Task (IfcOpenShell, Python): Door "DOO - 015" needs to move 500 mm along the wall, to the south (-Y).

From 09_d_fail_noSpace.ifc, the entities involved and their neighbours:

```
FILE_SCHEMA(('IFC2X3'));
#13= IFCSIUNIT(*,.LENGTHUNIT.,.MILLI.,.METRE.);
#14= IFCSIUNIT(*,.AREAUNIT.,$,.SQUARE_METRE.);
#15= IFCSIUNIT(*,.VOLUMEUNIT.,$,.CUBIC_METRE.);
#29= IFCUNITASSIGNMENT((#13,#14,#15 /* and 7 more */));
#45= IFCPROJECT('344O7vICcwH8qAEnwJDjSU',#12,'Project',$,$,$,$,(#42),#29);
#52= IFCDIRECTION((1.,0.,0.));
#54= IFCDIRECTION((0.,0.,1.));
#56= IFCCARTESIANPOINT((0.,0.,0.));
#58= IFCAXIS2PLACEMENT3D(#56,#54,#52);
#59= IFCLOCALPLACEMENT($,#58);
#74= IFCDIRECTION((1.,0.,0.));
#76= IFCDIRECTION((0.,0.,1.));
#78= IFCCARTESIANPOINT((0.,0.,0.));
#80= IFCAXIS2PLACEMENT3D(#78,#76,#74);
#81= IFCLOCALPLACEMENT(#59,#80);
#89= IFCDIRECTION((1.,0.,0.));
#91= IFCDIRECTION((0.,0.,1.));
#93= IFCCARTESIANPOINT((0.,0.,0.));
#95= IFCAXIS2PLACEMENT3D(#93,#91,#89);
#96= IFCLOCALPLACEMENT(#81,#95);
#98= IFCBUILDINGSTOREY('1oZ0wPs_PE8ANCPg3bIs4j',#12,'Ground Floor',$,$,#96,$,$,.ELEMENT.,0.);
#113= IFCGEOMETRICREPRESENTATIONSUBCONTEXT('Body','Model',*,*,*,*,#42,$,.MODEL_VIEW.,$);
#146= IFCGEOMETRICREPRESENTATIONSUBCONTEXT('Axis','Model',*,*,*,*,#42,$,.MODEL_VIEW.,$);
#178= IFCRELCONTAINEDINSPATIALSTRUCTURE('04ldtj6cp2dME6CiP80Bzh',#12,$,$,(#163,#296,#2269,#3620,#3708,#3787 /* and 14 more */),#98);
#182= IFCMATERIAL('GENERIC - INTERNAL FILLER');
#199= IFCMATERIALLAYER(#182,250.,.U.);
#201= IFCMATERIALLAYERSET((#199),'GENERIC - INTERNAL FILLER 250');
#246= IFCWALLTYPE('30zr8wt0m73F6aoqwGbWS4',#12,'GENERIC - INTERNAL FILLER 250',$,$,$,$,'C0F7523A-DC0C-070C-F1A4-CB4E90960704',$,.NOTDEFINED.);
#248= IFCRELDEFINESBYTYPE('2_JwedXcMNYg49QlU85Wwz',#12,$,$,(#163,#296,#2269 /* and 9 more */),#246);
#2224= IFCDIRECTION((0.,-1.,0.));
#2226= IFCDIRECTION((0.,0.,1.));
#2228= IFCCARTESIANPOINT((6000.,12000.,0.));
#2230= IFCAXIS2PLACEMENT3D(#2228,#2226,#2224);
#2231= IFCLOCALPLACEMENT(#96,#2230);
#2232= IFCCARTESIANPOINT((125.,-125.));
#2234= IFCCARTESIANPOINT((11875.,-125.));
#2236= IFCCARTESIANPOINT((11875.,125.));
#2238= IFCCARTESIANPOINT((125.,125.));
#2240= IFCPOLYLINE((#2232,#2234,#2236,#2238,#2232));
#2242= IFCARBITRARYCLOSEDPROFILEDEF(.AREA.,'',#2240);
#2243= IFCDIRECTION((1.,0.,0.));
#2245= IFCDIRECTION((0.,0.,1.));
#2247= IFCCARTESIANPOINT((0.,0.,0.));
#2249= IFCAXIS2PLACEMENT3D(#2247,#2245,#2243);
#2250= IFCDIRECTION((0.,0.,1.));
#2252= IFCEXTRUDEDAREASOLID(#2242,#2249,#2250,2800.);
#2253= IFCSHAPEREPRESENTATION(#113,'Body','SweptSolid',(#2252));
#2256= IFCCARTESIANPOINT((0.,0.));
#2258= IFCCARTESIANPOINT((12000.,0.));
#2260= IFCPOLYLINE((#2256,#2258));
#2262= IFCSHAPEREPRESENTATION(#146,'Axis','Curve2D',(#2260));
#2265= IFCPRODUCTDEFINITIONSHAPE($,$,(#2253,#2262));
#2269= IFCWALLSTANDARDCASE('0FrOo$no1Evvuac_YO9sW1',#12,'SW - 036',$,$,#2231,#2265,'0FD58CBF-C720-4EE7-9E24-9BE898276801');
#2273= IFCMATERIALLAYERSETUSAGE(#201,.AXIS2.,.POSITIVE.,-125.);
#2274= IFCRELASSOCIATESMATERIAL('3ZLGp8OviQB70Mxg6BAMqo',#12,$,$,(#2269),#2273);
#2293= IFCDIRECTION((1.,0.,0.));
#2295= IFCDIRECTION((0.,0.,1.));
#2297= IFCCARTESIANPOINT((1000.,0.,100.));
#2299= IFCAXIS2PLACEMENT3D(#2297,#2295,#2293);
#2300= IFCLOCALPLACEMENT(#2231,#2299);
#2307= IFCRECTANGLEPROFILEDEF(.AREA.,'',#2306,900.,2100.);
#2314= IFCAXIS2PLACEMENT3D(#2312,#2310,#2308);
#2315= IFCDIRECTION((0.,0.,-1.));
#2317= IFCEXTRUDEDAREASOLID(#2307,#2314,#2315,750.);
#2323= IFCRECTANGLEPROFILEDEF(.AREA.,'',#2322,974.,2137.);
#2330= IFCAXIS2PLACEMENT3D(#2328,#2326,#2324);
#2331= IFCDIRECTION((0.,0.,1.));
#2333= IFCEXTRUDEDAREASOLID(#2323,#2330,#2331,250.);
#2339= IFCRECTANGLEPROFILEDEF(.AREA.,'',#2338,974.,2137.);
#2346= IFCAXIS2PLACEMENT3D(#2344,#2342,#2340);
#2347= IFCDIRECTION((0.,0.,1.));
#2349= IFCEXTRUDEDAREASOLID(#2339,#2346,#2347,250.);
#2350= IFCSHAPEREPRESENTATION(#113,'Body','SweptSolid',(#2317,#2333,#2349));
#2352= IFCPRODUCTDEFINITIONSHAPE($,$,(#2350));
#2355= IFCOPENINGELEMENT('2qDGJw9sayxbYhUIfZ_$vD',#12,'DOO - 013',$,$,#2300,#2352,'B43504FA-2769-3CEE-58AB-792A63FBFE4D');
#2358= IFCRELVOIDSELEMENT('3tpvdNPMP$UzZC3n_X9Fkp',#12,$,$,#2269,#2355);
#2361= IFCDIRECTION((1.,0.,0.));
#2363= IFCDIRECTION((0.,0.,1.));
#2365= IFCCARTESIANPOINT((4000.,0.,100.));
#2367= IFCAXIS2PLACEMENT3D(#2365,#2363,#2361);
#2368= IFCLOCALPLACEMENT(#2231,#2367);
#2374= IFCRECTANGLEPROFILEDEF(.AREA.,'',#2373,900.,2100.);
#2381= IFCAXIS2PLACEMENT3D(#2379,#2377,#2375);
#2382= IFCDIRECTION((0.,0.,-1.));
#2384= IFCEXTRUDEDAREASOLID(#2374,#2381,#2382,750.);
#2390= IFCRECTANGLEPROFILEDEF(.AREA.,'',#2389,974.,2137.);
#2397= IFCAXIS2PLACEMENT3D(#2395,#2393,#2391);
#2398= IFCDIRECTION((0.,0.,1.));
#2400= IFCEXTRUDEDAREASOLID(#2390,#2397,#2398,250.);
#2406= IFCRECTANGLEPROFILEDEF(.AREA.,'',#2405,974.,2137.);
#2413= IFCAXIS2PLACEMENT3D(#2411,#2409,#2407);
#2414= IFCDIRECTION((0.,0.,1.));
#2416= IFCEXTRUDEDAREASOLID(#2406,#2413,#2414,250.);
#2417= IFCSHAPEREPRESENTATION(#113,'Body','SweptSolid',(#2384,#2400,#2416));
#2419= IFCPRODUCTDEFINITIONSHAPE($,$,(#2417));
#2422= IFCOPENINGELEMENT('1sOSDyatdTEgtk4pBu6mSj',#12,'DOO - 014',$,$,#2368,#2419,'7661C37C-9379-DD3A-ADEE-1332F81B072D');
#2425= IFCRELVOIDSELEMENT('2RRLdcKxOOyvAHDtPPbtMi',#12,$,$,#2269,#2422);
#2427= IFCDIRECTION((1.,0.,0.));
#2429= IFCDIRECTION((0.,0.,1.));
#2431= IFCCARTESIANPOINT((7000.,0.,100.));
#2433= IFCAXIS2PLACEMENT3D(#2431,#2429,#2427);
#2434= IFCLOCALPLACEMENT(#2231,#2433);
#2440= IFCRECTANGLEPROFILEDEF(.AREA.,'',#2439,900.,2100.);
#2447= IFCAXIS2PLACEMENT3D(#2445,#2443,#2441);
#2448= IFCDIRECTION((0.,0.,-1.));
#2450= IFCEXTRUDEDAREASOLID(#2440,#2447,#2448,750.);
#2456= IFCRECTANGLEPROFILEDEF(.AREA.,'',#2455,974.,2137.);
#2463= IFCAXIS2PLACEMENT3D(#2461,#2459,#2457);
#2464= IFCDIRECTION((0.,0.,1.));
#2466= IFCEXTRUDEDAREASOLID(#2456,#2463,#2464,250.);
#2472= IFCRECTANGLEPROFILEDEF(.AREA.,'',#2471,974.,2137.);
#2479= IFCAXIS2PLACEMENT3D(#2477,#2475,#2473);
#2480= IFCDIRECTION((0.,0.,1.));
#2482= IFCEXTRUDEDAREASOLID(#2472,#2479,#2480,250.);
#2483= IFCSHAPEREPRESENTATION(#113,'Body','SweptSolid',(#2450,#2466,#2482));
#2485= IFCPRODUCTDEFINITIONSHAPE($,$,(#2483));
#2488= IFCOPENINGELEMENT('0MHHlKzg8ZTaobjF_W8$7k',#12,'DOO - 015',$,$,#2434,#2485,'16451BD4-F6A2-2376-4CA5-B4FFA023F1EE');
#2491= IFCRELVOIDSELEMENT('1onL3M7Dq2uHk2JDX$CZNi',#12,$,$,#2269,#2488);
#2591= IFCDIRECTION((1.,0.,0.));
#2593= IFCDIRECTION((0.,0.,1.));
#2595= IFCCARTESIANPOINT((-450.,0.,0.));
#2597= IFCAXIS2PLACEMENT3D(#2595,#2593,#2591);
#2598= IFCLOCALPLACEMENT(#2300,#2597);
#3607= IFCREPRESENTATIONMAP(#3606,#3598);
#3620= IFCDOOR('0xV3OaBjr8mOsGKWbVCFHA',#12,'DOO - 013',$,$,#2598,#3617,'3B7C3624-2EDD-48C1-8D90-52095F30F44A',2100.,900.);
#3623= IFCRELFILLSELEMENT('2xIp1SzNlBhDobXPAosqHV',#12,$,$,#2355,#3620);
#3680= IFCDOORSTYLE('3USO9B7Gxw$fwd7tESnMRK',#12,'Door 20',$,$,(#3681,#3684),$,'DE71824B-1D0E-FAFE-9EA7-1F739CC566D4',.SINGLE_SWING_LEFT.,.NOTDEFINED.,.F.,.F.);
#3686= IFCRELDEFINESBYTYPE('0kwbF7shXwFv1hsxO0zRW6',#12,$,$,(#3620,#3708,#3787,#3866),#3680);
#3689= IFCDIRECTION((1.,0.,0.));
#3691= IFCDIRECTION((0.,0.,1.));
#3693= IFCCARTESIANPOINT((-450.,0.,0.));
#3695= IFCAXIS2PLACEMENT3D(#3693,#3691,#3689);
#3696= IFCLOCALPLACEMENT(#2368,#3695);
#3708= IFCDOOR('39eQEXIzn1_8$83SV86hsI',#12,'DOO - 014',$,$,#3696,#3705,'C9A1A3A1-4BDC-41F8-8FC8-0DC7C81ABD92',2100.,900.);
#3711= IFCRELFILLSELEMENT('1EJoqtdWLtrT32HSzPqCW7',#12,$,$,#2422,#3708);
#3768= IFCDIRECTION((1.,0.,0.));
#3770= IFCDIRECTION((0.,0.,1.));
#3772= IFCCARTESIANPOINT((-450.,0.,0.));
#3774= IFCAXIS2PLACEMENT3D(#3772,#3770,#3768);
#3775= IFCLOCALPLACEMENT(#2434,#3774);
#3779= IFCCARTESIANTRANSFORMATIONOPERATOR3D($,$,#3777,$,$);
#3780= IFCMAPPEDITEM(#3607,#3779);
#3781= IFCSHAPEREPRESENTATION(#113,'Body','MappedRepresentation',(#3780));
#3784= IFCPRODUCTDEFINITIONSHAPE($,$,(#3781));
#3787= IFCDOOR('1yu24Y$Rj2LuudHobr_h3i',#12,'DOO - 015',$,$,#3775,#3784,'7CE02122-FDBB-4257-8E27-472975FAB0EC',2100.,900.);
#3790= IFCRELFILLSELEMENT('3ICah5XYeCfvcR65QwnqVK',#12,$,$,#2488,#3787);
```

```python
import ifcopenshell
import ifcopenshell.api.geometry
import ifcopenshell.util.placement
import ifcopenshell.util.unit

model = ifcopenshell.open("09_d_fail_noSpace.ifc")
unit_scale = ifcopenshell.util.unit.calculate_unit_scale(model)

door = model.by_guid("1yu24Y$Rj2LuudHobr_h3i")
opening = door.FillsVoids[0].RelatingOpeningElement
wall = opening.VoidsElements[0].RelatingBuildingElement

wall_matrix = ifcopenshell.util.placement.get_local_placement(wall.ObjectPlacement)
shift = wall_matrix[:3, 0] * 0.5 / unit_scale
before = ifcopenshell.util.placement.get_local_placement(door.ObjectPlacement)[:3, 3].copy()

# The door is placed relative to its opening, so it follows when the opening moves.
matrix = ifcopenshell.util.placement.get_local_placement(opening.ObjectPlacement)
matrix[:3, 3] += shift
ifcopenshell.api.geometry.edit_object_placement(
    model, product=opening, matrix=matrix, is_si=False, should_transform_children=True
)

after = ifcopenshell.util.placement.get_local_placement(door.ObjectPlacement)[:3, 3]
print("door moved by", (after - before).round(3) + 0.0)

model.write("09_d_fail_noSpace_updated.ifc")
```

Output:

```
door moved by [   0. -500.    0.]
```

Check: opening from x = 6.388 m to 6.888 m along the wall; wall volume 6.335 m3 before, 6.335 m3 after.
